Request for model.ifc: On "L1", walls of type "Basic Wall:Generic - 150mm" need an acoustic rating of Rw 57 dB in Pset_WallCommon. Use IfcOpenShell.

First a look at what the model holds.

```python
import ifcopenshell
import ifcopenshell.util.element

model = ifcopenshell.open("model.ifc")
print(model.schema)
storey = next(s for s in model.by_type("IfcBuildingStorey") if s.Name == "L1")
walls = [e for e in ifcopenshell.util.element.get_decomposition(storey) if e.is_a("IfcWall")]
seen = {}
for e in walls:
    element_type = ifcopenshell.util.element.get_type(e)
    key = (element_type.Name if element_type != e and element_type else None, ifcopenshell.util.element.get_pset(e, "Pset_WallCommon", "AcousticRating"))
    seen[key] = seen.get(key, 0) + 1
for (name, value), count in sorted(seen.items(), key=str):
    print(count, "x", name, "|", value)
```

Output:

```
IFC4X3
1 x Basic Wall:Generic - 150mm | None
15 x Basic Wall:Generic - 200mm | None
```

```python
import ifcopenshell
import ifcopenshell.api.pset
import ifcopenshell.util.element

model = ifcopenshell.open("model.ifc")

storey = next(s for s in model.by_type("IfcBuildingStorey") if s.Name == "L1")
walls = [e for e in ifcopenshell.util.element.get_decomposition(storey) if e.is_a("IfcWall")]

count = 0
for e in walls:
    element_type = ifcopenshell.util.element.get_type(e)
    if element_type in (None, e) or element_type.Name != "Basic Wall:Generic - 150mm":
        continue
    # add_pset returns the element's existing set when there is one.
    pset = ifcopenshell.api.pset.add_pset(model, product=e, name="Pset_WallCommon")
    ifcopenshell.api.pset.edit_pset(model, pset=pset, properties={"AcousticRating": "Rw 57 dB"})
    count += 1

print(count, "walls updated")

model.write("model_edited.ifc")
```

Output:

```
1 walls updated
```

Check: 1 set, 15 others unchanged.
